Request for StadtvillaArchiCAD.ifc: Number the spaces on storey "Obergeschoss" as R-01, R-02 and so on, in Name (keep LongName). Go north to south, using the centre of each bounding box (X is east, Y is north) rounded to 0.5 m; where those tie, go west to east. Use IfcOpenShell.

First a look at what the model holds.

```python
import ifcopenshell
import ifcopenshell.util.element
import ifcopenshell.util.placement

model = ifcopenshell.open("StadtvillaArchiCAD.ifc")
print(model.schema)
storey = next(s for s in model.by_type("IfcBuildingStorey") if s.Name == "Obergeschoss")
spaces = [e for e in ifcopenshell.util.element.get_decomposition(storey) if e.is_a("IfcSpace")]
for e in sorted(spaces, key=lambda e: e.id()):
    origin = ifcopenshell.util.placement.get_local_placement(e.ObjectPlacement)[:3, 3]
    print(e.id(), e.Name, e.LongName, origin.round(2) + 0.0, sep=" | ")
```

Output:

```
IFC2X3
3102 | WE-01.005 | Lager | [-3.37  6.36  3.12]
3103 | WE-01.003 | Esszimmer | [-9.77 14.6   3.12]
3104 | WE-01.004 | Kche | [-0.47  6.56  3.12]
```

```python
import ifcopenshell
import ifcopenshell.geom
import ifcopenshell.util.element
import ifcopenshell.util.shape

model = ifcopenshell.open("StadtvillaArchiCAD.ifc")
settings = ifcopenshell.geom.settings()
settings.set("use-world-coords", True)


def centre(element):
    shape = ifcopenshell.geom.create_shape(settings, element)
    return ifcopenshell.util.shape.get_bbox_centroid(shape.geometry)


storey = next(s for s in model.by_type("IfcBuildingStorey") if s.Name == "Obergeschoss")
spaces = [e for e in ifcopenshell.util.element.get_decomposition(storey) if e.is_a("IfcSpace")]

# Insertion points can sit at a corner or the storey origin, so sort by the geometry (in metres).
centres = {e: centre(e) for e in spaces}
spaces.sort(key=lambda e: (-round(centres[e][1] / 0.5), centres[e][0]))

for i, e in enumerate(spaces, start=1):
    number = f"R-{i:02d}"
    e.Name = number
    print(e.id(), number)

model.write("StadtvillaArchiCAD_v2.ifc")
```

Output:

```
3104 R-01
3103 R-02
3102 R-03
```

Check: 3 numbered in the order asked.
